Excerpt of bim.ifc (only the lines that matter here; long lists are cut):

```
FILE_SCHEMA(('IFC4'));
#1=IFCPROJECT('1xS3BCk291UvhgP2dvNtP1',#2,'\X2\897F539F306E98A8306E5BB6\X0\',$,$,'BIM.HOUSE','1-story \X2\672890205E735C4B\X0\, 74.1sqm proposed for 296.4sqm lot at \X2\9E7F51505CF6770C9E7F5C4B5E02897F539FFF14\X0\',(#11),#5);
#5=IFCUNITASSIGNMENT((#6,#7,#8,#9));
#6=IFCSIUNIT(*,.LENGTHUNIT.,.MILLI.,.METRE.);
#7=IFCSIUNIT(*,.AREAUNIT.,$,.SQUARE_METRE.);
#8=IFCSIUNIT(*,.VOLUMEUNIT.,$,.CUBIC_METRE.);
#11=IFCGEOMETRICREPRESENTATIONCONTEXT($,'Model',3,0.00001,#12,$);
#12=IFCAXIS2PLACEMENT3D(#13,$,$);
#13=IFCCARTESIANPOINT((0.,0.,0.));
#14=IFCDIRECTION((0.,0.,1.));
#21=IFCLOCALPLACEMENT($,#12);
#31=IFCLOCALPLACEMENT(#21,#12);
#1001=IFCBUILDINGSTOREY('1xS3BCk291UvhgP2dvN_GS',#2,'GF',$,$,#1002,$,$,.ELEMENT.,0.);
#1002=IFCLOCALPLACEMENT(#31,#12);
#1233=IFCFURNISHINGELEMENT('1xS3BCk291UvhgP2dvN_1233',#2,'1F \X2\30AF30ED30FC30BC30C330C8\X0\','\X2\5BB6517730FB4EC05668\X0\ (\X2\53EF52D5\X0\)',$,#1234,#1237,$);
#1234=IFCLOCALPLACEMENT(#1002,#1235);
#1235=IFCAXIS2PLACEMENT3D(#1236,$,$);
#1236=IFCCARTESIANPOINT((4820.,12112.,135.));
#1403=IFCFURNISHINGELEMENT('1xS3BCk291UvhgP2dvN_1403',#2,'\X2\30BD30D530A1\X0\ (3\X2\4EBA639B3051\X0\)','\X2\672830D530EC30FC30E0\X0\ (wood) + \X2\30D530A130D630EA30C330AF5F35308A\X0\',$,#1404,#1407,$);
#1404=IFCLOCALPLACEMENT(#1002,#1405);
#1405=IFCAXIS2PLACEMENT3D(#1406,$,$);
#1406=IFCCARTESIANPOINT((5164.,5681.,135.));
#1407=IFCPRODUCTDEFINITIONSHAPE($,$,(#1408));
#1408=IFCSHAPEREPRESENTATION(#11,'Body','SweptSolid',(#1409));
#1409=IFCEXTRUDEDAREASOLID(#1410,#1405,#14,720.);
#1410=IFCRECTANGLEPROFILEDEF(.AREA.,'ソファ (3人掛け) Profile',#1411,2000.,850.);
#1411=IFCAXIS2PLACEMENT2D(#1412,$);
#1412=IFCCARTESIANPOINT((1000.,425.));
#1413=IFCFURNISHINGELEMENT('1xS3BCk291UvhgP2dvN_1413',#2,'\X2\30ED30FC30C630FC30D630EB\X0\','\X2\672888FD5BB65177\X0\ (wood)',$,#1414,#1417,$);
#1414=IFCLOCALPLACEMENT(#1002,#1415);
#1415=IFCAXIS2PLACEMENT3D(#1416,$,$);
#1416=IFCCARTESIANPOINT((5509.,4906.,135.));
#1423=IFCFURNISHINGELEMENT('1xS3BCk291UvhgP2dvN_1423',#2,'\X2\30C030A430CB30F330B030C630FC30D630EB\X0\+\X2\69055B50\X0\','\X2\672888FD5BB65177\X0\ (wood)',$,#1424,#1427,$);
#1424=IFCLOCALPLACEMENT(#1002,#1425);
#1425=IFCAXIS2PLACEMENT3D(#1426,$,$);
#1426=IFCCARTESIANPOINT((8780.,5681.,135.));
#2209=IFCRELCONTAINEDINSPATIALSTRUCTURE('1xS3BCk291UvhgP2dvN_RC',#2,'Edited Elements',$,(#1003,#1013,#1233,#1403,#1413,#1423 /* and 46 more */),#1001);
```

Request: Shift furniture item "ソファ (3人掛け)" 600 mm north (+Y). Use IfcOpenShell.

```python
import ifcopenshell
import ifcopenshell.api.geometry
import ifcopenshell.util.placement

model = ifcopenshell.open("bim.ifc")

item = model.by_guid("1xS3BCk291UvhgP2dvN_1403")
matrix = ifcopenshell.util.placement.get_local_placement(item.ObjectPlacement)
matrix[1, 3] += 600.0
ifcopenshell.api.geometry.edit_object_placement(model, product=item, matrix=matrix, is_si=False)

print(ifcopenshell.util.placement.get_local_placement(item.ObjectPlacement).round(3) + 0.0)

model.write("bim_rev.ifc")
```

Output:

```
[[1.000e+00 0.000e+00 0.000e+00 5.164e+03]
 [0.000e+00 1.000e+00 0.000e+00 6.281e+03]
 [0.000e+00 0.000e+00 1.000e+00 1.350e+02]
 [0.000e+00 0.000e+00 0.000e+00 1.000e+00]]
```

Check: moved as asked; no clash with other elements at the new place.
